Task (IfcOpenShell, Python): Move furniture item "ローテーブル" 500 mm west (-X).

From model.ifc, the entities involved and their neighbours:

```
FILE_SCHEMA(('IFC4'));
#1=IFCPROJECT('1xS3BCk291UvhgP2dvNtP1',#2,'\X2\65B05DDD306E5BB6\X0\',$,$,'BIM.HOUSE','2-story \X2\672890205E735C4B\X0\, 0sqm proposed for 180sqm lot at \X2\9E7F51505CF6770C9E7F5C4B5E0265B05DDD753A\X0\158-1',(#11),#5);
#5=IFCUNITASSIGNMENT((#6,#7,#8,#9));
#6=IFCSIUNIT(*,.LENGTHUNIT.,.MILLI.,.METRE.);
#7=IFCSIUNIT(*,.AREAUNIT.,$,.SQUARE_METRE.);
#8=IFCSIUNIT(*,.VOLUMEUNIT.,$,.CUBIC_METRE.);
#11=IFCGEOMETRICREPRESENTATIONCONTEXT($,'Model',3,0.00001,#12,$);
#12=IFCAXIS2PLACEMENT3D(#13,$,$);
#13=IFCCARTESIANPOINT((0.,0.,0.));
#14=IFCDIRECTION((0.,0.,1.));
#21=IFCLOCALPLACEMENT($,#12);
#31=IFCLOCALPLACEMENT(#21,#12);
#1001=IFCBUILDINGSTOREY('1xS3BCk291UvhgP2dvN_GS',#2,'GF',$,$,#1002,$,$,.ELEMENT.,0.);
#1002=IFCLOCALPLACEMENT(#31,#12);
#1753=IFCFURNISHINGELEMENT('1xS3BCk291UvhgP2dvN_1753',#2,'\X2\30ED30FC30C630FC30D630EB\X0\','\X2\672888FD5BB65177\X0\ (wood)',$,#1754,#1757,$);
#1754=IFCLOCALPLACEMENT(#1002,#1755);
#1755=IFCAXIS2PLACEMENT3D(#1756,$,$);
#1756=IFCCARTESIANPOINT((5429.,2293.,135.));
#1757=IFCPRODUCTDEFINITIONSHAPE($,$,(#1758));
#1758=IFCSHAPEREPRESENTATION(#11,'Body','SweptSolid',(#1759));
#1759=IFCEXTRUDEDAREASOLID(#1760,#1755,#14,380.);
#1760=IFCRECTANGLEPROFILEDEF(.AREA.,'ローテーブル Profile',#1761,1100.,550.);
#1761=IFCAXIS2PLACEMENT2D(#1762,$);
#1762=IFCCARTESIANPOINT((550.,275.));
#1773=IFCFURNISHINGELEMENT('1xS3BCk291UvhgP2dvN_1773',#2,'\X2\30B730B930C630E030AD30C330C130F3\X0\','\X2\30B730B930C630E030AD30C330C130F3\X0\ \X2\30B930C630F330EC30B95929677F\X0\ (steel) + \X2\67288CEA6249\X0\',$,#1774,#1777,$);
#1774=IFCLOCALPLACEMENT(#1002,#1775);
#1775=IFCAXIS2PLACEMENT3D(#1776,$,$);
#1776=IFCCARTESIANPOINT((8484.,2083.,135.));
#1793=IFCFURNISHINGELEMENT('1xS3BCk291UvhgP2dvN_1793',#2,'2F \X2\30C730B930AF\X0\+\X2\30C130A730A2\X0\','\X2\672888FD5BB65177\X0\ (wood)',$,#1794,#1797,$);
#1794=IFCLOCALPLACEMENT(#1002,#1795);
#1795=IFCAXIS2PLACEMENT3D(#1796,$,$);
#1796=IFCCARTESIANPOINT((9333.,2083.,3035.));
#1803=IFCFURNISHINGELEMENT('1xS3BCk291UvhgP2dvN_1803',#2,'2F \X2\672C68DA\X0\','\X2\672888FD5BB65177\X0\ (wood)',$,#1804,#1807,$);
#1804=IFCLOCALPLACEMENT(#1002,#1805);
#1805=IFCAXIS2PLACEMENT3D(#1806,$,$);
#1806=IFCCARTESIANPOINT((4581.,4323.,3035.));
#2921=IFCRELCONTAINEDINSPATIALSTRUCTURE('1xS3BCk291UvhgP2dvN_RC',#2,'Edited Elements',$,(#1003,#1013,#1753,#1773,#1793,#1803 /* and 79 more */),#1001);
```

```python
import ifcopenshell
import ifcopenshell.api.geometry
import ifcopenshell.util.placement
import ifcopenshell.util.unit

model = ifcopenshell.open("model.ifc")
unit_scale = ifcopenshell.util.unit.calculate_unit_scale(model)

item = model.by_guid("1xS3BCk291UvhgP2dvN_1753")
matrix = ifcopenshell.util.placement.get_local_placement(item.ObjectPlacement)
matrix[0, 3] -= 0.5 / unit_scale
ifcopenshell.api.geometry.edit_object_placement(model, product=item, matrix=matrix, is_si=False)

print(ifcopenshell.util.placement.get_local_placement(item.ObjectPlacement).round(3) + 0.0)

model.write("model_v2.ifc")
```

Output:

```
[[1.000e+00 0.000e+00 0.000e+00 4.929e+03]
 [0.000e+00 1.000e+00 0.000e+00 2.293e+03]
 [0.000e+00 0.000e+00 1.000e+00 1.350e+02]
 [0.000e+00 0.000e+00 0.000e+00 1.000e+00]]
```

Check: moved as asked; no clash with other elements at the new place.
